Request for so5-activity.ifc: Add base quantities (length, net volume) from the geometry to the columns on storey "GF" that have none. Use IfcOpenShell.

First a look at what the model holds.

```python
import ifcopenshell
import ifcopenshell.util.element
import ifcopenshell.util.unit

model = ifcopenshell.open("so5-activity.ifc")
print(model.schema)
for unit_type in ("LENGTHUNIT", "AREAUNIT", "VOLUMEUNIT"):
    print(unit_type, ifcopenshell.util.unit.calculate_unit_scale(model, unit_type))
storey = next(s for s in model.by_type("IfcBuildingStorey") if s.Name == "GF")
columns = [e for e in ifcopenshell.util.element.get_decomposition(storey) if e.is_a("IfcColumn")]
for e in sorted(columns, key=lambda e: e.id()):
    print(e.id(), e.is_a(), e.Name, list(ifcopenshell.util.element.get_psets(e, qtos_only=True)), sep=" | ")
```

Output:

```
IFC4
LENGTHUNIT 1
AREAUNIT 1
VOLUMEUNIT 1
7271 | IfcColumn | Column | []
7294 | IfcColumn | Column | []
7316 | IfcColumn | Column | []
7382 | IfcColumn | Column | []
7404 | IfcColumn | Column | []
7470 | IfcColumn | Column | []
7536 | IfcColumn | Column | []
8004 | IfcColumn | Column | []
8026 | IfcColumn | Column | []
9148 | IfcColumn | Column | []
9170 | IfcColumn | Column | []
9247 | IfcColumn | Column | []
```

```python
import ifcopenshell
import ifcopenshell.api.pset
import ifcopenshell.geom
import ifcopenshell.util.element
import ifcopenshell.util.shape
import ifcopenshell.util.unit

model = ifcopenshell.open("so5-activity.ifc")
unit_scale = ifcopenshell.util.unit.calculate_unit_scale(model)
volume_scale = ifcopenshell.util.unit.calculate_unit_scale(model, "VOLUMEUNIT")
settings = ifcopenshell.geom.settings()

storey = next(s for s in model.by_type("IfcBuildingStorey") if s.Name == "GF")
columns = [e for e in ifcopenshell.util.element.get_decomposition(storey) if e.is_a("IfcColumn")]

for e in sorted(columns, key=lambda e: e.id()):
    if ifcopenshell.util.element.get_psets(e, qtos_only=True, should_inherit=False):
        continue
    # Geometry comes back in metres, in the element's own axes.
    shape = ifcopenshell.geom.create_shape(settings, e)
    values = {
        "Length": ifcopenshell.util.shape.get_z(shape.geometry) / unit_scale,
        "NetVolume": ifcopenshell.util.shape.get_volume(shape.geometry) / volume_scale,
    }
    qto = ifcopenshell.api.pset.add_qto(model, product=e, name="Qto_ColumnBaseQuantities")
    ifcopenshell.api.pset.edit_qto(model, qto=qto, properties=values)
    print(e.id(), {k: round(v, 3) for k, v in values.items()})

model.write("so5-activity_v2.ifc")
```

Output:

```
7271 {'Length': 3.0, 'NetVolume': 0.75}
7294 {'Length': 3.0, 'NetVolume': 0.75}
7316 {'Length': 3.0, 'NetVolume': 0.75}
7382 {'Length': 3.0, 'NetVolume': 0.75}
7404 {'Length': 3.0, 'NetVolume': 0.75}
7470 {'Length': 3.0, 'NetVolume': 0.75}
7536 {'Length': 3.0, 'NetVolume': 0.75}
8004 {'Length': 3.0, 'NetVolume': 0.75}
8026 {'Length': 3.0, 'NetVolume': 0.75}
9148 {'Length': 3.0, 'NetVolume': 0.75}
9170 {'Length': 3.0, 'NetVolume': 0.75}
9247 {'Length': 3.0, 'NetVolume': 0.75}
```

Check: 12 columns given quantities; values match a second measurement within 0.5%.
